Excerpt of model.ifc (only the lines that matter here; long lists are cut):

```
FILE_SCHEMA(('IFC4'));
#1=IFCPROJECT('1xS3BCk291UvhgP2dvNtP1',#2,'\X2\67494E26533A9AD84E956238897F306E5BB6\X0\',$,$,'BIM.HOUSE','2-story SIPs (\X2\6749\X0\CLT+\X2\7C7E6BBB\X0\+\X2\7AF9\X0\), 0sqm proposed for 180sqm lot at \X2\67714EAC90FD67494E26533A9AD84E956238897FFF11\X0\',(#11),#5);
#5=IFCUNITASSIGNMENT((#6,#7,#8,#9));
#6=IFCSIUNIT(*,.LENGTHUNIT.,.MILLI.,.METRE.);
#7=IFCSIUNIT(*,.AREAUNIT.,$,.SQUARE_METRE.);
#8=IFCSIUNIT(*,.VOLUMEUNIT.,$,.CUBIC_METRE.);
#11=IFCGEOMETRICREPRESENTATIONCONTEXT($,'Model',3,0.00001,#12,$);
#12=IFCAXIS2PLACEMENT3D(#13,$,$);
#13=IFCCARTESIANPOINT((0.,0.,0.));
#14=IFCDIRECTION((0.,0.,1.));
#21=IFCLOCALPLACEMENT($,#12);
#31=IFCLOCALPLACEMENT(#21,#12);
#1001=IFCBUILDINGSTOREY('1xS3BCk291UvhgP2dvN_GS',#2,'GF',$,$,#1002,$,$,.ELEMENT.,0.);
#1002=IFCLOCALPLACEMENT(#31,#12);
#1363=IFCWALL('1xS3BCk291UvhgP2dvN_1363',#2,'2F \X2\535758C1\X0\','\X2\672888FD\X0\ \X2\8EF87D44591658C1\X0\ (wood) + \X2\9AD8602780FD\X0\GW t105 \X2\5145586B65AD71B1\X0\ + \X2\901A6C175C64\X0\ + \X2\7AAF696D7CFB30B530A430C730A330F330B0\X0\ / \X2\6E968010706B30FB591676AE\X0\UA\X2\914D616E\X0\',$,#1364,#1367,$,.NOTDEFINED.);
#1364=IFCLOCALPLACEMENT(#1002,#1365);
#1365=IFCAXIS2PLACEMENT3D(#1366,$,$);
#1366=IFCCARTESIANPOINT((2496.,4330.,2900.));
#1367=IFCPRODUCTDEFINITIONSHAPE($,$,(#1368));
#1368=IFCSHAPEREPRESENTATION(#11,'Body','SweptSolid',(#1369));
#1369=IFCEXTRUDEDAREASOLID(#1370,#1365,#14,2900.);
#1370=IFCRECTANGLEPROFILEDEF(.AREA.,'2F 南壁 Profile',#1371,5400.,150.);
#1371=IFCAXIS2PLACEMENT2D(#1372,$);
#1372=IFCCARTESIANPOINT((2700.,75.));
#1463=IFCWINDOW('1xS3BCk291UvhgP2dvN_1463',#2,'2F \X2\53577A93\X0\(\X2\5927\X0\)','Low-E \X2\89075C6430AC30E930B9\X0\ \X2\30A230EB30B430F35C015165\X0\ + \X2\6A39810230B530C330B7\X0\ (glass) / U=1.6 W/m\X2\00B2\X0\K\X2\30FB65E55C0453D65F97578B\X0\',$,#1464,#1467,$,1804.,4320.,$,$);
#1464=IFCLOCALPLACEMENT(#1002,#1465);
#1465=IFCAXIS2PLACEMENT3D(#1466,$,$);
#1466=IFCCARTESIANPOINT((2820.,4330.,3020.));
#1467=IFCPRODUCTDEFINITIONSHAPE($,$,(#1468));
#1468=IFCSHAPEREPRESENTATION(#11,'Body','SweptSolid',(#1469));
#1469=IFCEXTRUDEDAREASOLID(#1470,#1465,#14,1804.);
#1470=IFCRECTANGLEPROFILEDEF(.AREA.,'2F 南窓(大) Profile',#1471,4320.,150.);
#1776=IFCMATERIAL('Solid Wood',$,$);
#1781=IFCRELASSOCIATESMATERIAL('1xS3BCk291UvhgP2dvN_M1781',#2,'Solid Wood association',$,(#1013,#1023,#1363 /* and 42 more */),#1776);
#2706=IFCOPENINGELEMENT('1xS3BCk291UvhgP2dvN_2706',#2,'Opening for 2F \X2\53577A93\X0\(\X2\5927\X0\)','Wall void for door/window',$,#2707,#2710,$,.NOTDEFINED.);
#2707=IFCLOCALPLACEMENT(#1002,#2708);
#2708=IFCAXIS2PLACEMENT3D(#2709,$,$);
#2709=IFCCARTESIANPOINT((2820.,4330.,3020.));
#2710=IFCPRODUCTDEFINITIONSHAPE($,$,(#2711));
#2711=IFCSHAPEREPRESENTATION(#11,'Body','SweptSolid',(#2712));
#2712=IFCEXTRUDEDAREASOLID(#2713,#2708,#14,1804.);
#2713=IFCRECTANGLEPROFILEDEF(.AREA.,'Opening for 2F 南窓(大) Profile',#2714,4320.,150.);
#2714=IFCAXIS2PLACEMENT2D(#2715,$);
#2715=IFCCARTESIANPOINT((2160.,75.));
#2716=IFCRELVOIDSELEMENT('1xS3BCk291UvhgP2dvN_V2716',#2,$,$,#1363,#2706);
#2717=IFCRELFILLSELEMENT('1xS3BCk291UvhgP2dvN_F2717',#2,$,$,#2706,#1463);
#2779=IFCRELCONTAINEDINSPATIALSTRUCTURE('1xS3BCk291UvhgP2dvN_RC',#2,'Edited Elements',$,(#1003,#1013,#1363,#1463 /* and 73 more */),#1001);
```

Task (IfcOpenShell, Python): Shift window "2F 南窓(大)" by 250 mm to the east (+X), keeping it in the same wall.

```python
import ifcopenshell
import ifcopenshell.api.geometry
import ifcopenshell.util.placement
import ifcopenshell.util.unit

model = ifcopenshell.open("model.ifc")
unit_scale = ifcopenshell.util.unit.calculate_unit_scale(model)

window = model.by_guid("1xS3BCk291UvhgP2dvN_1463")
opening = window.FillsVoids[0].RelatingOpeningElement
wall = opening.VoidsElements[0].RelatingBuildingElement

wall_matrix = ifcopenshell.util.placement.get_local_placement(wall.ObjectPlacement)
shift = wall_matrix[:3, 0] * 0.25 / unit_scale
before = ifcopenshell.util.placement.get_local_placement(window.ObjectPlacement)[:3, 3].copy()

# The window is not placed relative to its opening, so move both.
for product in (opening, window):
    matrix = ifcopenshell.util.placement.get_local_placement(product.ObjectPlacement)
    matrix[:3, 3] += shift
    ifcopenshell.api.geometry.edit_object_placement(model, product=product, matrix=matrix, is_si=False)

after = ifcopenshell.util.placement.get_local_placement(window.ObjectPlacement)[:3, 3]
print("window moved by", (after - before).round(3) + 0.0)

model.write("model-out.ifc")
```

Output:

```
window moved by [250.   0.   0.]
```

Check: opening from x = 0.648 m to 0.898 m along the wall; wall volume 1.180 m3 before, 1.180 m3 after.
